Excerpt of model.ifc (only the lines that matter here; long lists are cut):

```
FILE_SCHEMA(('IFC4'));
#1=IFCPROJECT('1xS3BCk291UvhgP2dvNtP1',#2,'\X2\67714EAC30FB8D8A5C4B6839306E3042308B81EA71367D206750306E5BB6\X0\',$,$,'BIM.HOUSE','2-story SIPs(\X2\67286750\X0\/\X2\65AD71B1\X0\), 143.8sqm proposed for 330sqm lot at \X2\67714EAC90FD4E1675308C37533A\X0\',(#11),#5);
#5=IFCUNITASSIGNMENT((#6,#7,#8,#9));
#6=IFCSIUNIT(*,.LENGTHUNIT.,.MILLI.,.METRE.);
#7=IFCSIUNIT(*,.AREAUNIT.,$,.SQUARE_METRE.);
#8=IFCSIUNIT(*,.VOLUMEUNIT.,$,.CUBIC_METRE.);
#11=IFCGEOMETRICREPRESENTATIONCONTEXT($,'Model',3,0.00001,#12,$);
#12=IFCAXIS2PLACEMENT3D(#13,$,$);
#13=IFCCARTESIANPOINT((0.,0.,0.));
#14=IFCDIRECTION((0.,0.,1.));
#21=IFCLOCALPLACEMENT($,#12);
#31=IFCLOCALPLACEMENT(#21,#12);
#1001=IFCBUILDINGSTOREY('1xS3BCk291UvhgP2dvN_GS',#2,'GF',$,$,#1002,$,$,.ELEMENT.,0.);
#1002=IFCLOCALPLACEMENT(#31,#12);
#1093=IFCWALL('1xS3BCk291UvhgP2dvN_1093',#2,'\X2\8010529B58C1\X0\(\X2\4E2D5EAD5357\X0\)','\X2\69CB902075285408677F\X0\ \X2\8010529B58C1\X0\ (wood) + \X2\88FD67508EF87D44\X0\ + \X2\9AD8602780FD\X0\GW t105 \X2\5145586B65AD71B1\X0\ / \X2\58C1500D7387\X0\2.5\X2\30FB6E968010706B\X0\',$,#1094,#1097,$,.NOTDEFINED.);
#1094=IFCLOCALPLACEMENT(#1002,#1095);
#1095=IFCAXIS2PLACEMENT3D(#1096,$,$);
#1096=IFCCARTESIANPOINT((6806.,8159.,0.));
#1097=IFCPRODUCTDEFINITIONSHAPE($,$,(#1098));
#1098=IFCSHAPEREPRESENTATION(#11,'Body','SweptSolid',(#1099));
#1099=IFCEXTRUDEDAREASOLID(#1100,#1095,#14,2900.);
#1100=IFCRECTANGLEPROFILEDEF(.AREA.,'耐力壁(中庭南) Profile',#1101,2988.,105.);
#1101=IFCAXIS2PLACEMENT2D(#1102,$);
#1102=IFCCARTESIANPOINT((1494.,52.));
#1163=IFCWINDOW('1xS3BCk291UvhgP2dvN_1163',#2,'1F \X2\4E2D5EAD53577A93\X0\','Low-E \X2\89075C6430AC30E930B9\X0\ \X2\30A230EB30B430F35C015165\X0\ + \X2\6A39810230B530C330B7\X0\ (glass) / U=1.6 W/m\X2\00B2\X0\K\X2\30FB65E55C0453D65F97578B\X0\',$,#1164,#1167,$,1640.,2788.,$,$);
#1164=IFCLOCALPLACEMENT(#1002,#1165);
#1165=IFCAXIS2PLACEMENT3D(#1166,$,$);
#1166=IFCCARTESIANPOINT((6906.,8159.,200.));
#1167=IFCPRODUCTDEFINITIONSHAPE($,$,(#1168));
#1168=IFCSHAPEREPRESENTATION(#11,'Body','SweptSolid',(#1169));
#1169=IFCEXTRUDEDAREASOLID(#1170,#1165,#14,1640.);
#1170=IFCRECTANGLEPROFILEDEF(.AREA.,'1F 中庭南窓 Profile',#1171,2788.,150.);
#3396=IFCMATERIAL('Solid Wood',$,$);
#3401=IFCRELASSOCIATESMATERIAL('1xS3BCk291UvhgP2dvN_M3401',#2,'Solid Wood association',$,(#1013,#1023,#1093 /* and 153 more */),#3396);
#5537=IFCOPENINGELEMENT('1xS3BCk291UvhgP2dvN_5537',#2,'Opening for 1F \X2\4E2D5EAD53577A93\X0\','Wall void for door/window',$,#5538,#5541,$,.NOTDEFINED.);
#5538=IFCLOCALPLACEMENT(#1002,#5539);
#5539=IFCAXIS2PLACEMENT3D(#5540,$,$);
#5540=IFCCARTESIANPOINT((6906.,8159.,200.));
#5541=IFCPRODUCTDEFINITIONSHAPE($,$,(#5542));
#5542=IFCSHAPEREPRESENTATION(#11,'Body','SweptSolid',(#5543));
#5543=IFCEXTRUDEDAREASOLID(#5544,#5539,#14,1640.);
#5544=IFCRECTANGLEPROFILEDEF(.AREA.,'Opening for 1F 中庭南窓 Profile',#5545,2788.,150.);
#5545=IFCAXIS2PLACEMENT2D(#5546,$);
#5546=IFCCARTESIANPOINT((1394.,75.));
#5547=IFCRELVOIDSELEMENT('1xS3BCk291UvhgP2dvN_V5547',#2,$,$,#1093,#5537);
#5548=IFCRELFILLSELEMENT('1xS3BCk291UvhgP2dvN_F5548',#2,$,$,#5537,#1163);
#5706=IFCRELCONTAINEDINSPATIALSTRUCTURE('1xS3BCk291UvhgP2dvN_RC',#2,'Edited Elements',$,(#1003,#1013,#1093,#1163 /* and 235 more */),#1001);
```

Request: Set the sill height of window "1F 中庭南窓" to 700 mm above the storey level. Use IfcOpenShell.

```python
import numpy as np
import ifcopenshell
import ifcopenshell.api.geometry
import ifcopenshell.geom
import ifcopenshell.util.element
import ifcopenshell.util.placement
import ifcopenshell.util.shape
import ifcopenshell.util.unit

model = ifcopenshell.open("model.ifc")
unit_scale = ifcopenshell.util.unit.calculate_unit_scale(model)

window = model.by_guid("1xS3BCk291UvhgP2dvN_1163")
opening = window.FillsVoids[0].RelatingOpeningElement
storey = ifcopenshell.util.element.get_container(window, ifc_class="IfcBuildingStorey")
level = ifcopenshell.util.placement.get_local_placement(storey.ObjectPlacement)[2, 3]

# The opening's origin need not be at the sill, so measure its lowest point.
shape = ifcopenshell.geom.create_shape(ifcopenshell.geom.settings(), opening)
bottom = ifcopenshell.util.shape.get_shape_bottom_elevation(shape, shape.geometry) / unit_scale
dz = level + 0.7 / unit_scale - bottom

shift = np.array([0.0, 0.0, dz])
# The window is not placed relative to its opening, so move both.
for product in (opening, window):
    matrix = ifcopenshell.util.placement.get_local_placement(product.ObjectPlacement)
    matrix[:3, 3] += shift
    ifcopenshell.api.geometry.edit_object_placement(model, product=product, matrix=matrix, is_si=False)

print(f"moved by {dz * unit_scale:+.3f} m")

model.write("model_updated.ifc")
```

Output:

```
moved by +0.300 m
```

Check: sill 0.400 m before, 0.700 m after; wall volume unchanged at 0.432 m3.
